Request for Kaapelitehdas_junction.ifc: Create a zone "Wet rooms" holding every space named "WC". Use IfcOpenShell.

First a look at what the model holds.

```python
import ifcopenshell

model = ifcopenshell.open("Kaapelitehdas_junction.ifc")
print(model.schema)
seen = {}
for space in model.by_type("IfcSpace"):
    seen[space.LongName] = seen.get(space.LongName, 0) + 1
for name, count in sorted(seen.items(), key=str):
    print(count, "x", name)
print("zones:", [z.Name for z in model.by_type("IfcZone")][:20])
```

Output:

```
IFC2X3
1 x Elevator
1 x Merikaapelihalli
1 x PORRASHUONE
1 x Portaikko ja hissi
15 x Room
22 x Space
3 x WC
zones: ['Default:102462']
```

```python
import ifcopenshell
import ifcopenshell.api.group
import ifcopenshell.api.root

model = ifcopenshell.open("Kaapelitehdas_junction.ifc")

names = {"WC"}
spaces = [s for s in model.by_type("IfcSpace") if s.LongName in names]

zone = ifcopenshell.api.root.create_entity(model, ifc_class="IfcZone", name="Wet rooms")
ifcopenshell.api.group.assign_group(model, products=spaces, group=zone)
print(len(spaces), "spaces in", zone.Name)

model.write("Kaapelitehdas_junction_v2.ifc")
```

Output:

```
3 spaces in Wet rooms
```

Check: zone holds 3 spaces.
